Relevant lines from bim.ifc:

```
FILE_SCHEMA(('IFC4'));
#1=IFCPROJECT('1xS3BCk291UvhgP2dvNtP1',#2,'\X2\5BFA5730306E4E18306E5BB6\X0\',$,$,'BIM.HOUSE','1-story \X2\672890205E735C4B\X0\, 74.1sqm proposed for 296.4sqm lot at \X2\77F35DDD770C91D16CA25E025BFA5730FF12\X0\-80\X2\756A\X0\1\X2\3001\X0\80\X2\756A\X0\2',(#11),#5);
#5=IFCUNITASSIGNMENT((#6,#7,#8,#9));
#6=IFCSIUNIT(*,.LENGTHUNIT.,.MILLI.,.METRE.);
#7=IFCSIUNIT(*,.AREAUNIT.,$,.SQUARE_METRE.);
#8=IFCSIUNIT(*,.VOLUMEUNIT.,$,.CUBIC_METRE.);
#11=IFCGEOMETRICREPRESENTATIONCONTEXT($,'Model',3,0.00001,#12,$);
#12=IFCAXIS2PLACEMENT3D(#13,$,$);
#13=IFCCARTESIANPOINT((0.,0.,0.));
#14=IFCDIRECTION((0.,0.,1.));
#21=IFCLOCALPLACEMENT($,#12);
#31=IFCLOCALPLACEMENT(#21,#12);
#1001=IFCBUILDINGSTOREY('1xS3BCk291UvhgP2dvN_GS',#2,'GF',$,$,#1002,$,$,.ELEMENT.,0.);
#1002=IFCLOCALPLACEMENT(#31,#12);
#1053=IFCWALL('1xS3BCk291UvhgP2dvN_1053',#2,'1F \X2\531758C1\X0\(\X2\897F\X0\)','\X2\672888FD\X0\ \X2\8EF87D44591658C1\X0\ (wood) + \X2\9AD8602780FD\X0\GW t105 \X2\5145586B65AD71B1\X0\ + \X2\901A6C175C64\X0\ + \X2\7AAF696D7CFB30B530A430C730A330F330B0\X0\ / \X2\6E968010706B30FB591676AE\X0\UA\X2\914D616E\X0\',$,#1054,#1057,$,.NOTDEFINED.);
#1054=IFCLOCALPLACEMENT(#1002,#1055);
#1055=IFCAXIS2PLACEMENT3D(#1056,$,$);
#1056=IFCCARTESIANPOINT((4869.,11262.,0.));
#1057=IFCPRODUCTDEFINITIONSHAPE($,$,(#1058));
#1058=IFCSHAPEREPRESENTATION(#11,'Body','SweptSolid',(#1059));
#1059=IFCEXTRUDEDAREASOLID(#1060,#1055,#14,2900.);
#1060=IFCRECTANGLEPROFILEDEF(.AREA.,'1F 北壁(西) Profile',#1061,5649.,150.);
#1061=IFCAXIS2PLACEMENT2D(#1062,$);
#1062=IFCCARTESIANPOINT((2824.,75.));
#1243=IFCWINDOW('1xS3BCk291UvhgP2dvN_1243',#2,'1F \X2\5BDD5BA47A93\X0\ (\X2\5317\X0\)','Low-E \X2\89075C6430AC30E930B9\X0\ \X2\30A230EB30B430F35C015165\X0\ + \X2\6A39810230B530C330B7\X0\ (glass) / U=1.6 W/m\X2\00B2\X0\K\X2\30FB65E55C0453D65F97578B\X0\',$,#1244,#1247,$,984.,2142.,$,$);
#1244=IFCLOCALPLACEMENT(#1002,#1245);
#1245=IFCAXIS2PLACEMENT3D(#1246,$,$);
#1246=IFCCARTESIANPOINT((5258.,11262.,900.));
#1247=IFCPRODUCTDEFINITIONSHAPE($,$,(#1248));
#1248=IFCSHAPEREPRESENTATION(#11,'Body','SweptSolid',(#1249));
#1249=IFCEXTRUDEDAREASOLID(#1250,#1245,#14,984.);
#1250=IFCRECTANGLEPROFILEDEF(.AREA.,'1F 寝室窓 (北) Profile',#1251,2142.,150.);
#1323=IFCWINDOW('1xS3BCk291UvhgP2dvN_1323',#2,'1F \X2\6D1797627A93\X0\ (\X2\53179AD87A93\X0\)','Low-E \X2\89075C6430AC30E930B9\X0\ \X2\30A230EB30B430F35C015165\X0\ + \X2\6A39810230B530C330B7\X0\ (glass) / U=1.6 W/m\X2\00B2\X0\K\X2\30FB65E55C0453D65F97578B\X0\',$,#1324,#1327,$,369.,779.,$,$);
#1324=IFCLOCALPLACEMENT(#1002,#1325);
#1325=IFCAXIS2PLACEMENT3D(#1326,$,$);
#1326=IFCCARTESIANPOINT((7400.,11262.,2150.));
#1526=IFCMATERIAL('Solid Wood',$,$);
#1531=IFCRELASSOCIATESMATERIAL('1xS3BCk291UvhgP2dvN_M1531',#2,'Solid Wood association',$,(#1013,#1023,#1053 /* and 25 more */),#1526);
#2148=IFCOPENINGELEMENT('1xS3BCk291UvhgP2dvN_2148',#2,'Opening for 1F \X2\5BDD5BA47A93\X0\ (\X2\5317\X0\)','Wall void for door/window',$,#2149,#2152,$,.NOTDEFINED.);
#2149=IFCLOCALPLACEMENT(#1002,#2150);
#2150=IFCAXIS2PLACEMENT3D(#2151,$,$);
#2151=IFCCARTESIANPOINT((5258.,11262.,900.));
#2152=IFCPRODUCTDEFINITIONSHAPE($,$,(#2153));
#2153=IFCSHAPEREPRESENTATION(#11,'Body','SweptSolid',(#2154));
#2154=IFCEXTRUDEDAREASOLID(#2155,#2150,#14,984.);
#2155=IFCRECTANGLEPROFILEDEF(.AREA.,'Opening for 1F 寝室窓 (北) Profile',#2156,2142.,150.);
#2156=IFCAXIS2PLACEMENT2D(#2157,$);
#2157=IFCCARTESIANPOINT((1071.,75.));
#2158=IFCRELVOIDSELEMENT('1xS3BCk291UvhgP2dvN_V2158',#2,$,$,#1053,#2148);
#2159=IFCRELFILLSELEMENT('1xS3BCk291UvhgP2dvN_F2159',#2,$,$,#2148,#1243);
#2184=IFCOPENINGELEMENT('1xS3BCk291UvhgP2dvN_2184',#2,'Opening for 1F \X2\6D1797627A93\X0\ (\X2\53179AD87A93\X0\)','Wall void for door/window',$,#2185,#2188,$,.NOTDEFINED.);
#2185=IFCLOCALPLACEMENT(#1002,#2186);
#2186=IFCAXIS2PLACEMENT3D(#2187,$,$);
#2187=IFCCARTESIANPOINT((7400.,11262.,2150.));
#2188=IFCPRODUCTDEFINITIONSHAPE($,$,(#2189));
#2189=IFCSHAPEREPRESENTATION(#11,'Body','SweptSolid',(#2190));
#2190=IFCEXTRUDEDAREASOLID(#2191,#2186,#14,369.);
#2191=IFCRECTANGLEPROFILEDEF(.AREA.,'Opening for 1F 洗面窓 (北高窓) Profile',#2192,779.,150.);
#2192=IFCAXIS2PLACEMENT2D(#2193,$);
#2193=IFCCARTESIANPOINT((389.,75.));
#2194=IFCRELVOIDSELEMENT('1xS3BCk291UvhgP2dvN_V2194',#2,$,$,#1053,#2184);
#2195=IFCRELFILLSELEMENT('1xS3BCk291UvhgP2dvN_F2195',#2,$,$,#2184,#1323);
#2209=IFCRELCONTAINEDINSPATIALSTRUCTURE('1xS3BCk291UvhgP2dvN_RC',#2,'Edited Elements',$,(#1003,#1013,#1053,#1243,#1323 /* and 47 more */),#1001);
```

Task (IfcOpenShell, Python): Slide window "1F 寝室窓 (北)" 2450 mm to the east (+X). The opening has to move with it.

```python
import ifcopenshell
import ifcopenshell.api.geometry
import ifcopenshell.util.placement
import ifcopenshell.util.unit

model = ifcopenshell.open("bim.ifc")
unit_scale = ifcopenshell.util.unit.calculate_unit_scale(model)

window = model.by_id(1243)
opening = window.FillsVoids[0].RelatingOpeningElement
wall = opening.VoidsElements[0].RelatingBuildingElement

wall_matrix = ifcopenshell.util.placement.get_local_placement(wall.ObjectPlacement)
shift = wall_matrix[:3, 0] * 2.45 / unit_scale
before = ifcopenshell.util.placement.get_local_placement(window.ObjectPlacement)[:3, 3].copy()

# The window is not placed relative to its opening, so move both.
for product in (opening, window):
    matrix = ifcopenshell.util.placement.get_local_placement(product.ObjectPlacement)
    matrix[:3, 3] += shift
    ifcopenshell.api.geometry.edit_object_placement(model, product=product, matrix=matrix, is_si=False)

after = ifcopenshell.util.placement.get_local_placement(window.ObjectPlacement)[:3, 3]
print("window moved by", (after - before).round(3) + 0.0)

model.write("bim_v2.ifc")
```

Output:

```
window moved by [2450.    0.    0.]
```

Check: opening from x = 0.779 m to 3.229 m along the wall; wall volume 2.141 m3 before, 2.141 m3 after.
